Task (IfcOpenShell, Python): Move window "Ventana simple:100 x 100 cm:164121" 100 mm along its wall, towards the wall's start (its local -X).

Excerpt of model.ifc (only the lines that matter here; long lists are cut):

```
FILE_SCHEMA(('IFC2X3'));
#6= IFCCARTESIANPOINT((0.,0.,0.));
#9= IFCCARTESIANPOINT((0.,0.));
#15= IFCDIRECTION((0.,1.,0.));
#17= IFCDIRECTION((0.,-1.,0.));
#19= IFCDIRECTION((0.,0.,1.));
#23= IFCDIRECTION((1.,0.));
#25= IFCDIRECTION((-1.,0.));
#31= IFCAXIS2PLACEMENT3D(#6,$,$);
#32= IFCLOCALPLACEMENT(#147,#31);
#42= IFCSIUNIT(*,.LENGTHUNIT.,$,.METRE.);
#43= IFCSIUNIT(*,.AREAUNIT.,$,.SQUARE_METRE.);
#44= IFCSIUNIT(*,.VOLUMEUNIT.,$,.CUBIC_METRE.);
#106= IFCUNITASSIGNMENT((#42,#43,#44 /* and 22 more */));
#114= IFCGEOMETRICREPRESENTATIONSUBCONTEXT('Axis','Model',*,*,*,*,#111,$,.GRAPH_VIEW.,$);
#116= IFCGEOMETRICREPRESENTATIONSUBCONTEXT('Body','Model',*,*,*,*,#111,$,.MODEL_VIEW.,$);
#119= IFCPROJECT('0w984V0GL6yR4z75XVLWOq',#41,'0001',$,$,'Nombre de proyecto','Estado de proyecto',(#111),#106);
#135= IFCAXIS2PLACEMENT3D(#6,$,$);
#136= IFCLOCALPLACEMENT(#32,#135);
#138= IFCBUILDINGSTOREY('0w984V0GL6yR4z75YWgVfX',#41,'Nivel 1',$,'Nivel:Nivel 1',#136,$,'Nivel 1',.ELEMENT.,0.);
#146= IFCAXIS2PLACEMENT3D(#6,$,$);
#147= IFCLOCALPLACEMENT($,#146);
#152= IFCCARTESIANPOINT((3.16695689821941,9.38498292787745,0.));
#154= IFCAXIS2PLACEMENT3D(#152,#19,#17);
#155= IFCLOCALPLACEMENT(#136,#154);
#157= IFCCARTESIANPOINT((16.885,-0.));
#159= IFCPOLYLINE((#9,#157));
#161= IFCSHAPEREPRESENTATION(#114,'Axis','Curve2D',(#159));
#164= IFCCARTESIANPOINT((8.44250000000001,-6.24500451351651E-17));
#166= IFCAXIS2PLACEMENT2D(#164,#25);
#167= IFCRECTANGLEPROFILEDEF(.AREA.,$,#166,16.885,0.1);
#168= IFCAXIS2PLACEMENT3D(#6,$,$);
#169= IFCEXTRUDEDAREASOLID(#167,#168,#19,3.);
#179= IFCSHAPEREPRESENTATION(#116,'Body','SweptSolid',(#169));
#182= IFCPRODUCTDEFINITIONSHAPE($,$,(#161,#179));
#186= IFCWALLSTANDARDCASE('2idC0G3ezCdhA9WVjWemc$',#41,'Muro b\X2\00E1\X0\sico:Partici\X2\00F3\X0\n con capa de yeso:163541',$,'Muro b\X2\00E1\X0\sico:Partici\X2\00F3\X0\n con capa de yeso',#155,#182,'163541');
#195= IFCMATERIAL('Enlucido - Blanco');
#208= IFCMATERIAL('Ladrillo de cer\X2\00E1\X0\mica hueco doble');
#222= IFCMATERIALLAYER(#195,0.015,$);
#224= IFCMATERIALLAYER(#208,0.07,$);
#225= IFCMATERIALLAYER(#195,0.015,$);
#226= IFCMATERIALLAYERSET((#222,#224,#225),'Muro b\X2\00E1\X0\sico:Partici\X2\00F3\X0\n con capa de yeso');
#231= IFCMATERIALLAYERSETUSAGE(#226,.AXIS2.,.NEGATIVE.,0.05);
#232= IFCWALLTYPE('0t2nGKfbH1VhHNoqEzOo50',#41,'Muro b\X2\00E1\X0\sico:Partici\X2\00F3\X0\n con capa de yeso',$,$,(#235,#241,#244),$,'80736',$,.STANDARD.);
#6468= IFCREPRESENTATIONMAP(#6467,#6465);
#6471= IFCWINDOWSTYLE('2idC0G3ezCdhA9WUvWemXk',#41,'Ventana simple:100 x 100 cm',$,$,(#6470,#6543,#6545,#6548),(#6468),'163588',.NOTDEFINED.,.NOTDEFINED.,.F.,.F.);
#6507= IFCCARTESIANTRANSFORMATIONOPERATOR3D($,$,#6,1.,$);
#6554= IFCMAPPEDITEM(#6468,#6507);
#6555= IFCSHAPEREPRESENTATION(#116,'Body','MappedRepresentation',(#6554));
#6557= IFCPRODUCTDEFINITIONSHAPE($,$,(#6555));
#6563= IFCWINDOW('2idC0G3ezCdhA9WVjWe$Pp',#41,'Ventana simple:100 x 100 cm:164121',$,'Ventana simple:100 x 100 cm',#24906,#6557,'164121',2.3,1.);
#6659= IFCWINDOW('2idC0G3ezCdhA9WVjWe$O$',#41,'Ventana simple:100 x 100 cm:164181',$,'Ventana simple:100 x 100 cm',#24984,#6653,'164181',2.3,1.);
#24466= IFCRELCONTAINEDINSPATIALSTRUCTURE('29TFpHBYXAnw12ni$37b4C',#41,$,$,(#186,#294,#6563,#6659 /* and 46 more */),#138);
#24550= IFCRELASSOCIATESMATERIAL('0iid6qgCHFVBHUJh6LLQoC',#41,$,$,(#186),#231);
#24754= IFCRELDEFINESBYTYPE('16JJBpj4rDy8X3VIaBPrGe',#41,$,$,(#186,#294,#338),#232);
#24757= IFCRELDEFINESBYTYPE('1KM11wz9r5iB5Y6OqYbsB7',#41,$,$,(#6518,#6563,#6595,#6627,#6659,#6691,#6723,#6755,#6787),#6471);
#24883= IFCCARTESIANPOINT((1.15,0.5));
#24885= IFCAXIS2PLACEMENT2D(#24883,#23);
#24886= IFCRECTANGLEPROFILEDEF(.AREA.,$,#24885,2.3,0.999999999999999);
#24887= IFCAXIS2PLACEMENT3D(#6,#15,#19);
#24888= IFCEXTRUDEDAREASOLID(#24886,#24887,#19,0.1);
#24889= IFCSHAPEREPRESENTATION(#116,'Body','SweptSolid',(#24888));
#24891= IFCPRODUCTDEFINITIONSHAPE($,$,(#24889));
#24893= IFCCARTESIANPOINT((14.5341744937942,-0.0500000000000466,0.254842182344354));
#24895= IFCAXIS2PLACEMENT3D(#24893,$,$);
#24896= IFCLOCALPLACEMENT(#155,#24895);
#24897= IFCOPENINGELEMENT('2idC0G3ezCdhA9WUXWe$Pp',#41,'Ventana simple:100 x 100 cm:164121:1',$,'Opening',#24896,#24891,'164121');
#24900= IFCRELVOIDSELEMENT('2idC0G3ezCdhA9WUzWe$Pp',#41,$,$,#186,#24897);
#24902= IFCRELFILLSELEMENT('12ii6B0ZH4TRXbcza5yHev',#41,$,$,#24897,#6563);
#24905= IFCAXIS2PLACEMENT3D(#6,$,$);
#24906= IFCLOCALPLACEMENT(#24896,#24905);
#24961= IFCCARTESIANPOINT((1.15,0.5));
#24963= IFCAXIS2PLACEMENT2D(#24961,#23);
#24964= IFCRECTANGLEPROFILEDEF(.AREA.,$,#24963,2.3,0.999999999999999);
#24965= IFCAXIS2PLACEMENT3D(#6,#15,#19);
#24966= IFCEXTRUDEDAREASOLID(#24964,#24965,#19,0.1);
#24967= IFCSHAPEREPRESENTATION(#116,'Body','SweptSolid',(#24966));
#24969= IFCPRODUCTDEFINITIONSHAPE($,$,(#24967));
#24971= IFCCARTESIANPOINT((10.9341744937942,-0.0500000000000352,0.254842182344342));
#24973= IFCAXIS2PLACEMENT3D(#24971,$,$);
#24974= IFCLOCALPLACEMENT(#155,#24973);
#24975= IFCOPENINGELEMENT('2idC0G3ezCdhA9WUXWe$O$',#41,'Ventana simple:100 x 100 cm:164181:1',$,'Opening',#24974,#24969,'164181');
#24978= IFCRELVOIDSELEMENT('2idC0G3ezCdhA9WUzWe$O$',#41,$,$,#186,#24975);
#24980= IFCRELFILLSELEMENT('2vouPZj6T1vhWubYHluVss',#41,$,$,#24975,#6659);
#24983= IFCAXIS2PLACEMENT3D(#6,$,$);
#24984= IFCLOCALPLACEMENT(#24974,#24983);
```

```python
import ifcopenshell
import ifcopenshell.api.geometry
import ifcopenshell.util.placement

model = ifcopenshell.open("model.ifc")

window = model.by_guid("2idC0G3ezCdhA9WVjWe$Pp")
opening = window.FillsVoids[0].RelatingOpeningElement
wall = opening.VoidsElements[0].RelatingBuildingElement

wall_matrix = ifcopenshell.util.placement.get_local_placement(wall.ObjectPlacement)
shift = wall_matrix[:3, 0] * -0.1
before = ifcopenshell.util.placement.get_local_placement(window.ObjectPlacement)[:3, 3].copy()

# The window is placed relative to its opening, so it follows when the opening moves.
matrix = ifcopenshell.util.placement.get_local_placement(opening.ObjectPlacement)
matrix[:3, 3] += shift
ifcopenshell.api.geometry.edit_object_placement(
    model, product=opening, matrix=matrix, is_si=False, should_transform_children=True
)

after = ifcopenshell.util.placement.get_local_placement(window.ObjectPlacement)[:3, 3]
print("window moved by", (after - before).round(3) + 0.0)

model.write("model_updated.ifc")
```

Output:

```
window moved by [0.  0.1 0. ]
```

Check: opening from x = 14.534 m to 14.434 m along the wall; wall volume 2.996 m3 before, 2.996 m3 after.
